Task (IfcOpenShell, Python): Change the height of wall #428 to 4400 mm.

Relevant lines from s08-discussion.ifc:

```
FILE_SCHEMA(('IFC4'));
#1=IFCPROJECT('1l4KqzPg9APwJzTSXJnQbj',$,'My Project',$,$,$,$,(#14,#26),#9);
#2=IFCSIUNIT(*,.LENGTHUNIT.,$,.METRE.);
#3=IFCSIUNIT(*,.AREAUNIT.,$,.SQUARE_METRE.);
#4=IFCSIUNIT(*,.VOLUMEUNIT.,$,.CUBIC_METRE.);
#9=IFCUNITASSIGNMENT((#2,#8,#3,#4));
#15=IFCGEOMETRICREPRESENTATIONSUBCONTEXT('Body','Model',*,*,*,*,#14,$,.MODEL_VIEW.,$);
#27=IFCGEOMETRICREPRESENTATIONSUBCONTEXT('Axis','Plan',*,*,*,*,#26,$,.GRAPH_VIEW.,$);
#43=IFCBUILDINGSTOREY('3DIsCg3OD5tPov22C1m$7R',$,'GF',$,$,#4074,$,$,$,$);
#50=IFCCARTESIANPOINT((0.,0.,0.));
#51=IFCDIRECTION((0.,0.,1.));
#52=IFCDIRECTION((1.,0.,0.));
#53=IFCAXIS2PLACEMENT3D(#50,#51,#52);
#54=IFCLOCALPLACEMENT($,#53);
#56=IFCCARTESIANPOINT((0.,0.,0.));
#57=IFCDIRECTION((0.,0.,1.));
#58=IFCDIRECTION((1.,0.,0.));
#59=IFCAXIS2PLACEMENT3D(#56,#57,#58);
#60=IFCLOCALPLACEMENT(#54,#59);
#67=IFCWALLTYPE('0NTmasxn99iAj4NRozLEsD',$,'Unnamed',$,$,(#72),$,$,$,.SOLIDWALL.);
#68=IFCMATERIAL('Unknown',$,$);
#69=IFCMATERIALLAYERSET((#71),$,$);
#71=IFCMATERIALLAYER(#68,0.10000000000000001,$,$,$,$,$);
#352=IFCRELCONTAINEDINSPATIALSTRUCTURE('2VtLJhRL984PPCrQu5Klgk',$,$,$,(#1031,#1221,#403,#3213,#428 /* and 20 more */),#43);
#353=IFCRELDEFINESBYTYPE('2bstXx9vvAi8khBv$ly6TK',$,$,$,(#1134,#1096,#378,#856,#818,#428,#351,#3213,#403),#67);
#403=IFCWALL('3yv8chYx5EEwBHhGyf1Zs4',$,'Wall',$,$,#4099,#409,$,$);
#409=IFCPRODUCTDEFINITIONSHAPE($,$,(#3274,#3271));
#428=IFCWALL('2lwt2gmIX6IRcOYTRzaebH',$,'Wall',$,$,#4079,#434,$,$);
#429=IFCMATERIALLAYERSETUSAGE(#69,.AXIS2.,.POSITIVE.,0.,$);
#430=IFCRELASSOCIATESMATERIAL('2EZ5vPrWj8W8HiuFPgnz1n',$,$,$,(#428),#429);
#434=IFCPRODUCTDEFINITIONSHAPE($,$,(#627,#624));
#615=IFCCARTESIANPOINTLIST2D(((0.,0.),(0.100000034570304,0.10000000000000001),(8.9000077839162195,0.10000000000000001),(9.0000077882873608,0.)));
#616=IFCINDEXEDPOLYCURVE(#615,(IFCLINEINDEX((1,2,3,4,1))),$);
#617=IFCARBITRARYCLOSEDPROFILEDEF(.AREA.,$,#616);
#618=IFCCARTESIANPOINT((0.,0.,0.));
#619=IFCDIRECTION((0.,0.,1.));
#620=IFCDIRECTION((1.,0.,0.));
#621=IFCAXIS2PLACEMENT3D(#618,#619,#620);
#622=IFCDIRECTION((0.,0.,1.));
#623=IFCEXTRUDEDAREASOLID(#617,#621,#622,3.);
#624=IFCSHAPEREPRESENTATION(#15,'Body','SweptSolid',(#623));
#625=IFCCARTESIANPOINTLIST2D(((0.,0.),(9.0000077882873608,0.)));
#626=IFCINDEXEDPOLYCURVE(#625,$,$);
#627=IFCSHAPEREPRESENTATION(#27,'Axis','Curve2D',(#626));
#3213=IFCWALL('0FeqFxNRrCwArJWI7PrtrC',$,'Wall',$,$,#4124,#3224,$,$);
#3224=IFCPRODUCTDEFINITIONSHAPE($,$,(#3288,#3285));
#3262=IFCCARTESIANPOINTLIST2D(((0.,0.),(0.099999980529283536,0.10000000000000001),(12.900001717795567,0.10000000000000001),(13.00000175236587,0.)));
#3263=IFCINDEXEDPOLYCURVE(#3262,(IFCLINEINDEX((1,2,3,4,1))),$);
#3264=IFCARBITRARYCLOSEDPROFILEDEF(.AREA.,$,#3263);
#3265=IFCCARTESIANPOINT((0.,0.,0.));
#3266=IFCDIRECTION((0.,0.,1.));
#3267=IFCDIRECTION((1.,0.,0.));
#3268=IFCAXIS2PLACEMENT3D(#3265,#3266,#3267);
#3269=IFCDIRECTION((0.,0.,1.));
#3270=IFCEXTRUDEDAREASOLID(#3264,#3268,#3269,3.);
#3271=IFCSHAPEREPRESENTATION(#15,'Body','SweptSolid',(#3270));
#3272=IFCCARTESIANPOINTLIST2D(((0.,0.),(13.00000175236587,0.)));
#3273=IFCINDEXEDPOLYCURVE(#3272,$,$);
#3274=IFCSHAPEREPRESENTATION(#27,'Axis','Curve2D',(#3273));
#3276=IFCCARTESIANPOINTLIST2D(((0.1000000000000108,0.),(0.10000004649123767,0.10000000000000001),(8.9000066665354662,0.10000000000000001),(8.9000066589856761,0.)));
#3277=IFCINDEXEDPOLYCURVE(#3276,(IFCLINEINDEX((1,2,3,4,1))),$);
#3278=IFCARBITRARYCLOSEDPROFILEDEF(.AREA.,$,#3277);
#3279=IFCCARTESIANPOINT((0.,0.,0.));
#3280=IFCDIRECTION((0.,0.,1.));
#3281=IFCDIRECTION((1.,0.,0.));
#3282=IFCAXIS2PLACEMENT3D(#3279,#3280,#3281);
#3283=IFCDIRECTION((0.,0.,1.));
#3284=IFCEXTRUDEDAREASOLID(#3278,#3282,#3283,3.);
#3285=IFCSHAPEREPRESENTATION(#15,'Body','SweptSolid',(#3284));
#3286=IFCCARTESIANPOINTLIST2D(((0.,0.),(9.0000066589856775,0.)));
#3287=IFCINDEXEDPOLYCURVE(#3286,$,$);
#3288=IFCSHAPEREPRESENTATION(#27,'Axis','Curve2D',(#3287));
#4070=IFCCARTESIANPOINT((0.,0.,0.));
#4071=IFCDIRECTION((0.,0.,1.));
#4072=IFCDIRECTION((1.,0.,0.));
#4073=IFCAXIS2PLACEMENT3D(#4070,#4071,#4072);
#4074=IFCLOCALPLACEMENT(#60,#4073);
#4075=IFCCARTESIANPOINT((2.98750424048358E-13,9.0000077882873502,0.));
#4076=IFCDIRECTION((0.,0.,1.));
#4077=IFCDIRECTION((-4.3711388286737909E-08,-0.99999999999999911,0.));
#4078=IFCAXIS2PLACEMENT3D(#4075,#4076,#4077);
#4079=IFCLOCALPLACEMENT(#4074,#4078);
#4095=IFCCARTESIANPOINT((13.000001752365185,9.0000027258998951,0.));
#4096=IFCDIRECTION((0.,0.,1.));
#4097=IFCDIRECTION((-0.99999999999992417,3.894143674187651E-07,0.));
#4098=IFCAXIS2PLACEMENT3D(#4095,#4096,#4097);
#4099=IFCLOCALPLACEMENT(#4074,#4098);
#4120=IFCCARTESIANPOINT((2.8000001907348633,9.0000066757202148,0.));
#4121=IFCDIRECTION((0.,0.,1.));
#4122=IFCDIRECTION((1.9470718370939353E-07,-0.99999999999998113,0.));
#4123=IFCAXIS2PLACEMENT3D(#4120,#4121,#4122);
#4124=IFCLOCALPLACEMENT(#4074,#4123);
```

```python
import ifcopenshell
import ifcopenshell.geom
import ifcopenshell.util.representation
import ifcopenshell.util.shape
import ifcopenshell.util.unit

model = ifcopenshell.open("s08-discussion.ifc")
unit_scale = ifcopenshell.util.unit.calculate_unit_scale(model)
settings = ifcopenshell.geom.settings()


def volume(element):
    """Net volume in cubic metres, openings subtracted."""
    shape = ifcopenshell.geom.create_shape(settings, element)
    return ifcopenshell.util.shape.get_volume(shape.geometry)


wall = model.by_id(428)
before = volume(wall)

body = ifcopenshell.util.representation.get_representation(wall, "Model", "Body")
solid = body.Items[0]
old_height = solid.Depth
solid.Depth = 4.4 / unit_scale
after = volume(wall)

print(f"height {old_height:g} -> {solid.Depth:g}, volume {before:.3f} -> {after:.3f} m3")

model.write("s08-discussion-out.ifc")
```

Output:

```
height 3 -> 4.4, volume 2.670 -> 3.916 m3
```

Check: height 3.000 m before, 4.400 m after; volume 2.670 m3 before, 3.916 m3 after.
